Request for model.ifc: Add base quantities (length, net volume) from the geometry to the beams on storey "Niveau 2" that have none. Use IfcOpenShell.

First a look at what the model holds.

```python
import ifcopenshell
import ifcopenshell.util.element
import ifcopenshell.util.unit

model = ifcopenshell.open("model.ifc")
print(model.schema)
for unit_type in ("LENGTHUNIT", "AREAUNIT", "VOLUMEUNIT"):
    print(unit_type, ifcopenshell.util.unit.calculate_unit_scale(model, unit_type))
storey = next(s for s in model.by_type("IfcBuildingStorey") if s.Name == "Niveau 2")
beams = [e for e in ifcopenshell.util.element.get_decomposition(storey) if e.is_a("IfcBeam")]
for e in sorted(beams, key=lambda e: e.id()):
    print(e.id(), e.is_a(), e.Name, list(ifcopenshell.util.element.get_psets(e, qtos_only=True)), sep=" | ")
```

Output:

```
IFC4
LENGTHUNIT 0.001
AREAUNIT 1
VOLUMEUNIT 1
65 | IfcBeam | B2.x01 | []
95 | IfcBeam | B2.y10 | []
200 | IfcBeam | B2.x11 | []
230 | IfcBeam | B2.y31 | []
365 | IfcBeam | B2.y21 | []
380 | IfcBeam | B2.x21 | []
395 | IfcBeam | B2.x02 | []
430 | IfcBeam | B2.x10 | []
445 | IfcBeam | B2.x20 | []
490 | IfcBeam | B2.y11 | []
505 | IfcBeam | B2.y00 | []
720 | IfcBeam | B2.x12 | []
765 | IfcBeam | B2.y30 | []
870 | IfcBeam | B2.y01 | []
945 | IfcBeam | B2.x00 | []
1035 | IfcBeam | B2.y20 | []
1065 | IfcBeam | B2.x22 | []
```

```python
import ifcopenshell
import ifcopenshell.api.pset
import ifcopenshell.geom
import ifcopenshell.util.element
import ifcopenshell.util.shape
import ifcopenshell.util.unit

model = ifcopenshell.open("model.ifc")
unit_scale = ifcopenshell.util.unit.calculate_unit_scale(model)
volume_scale = ifcopenshell.util.unit.calculate_unit_scale(model, "VOLUMEUNIT")
settings = ifcopenshell.geom.settings()

storey = next(s for s in model.by_type("IfcBuildingStorey") if s.Name == "Niveau 2")
beams = [e for e in ifcopenshell.util.element.get_decomposition(storey) if e.is_a("IfcBeam")]

for e in sorted(beams, key=lambda e: e.id()):
    if ifcopenshell.util.element.get_psets(e, qtos_only=True, should_inherit=False):
        continue
    # Geometry comes back in metres, in the element's own axes.
    shape = ifcopenshell.geom.create_shape(settings, e)
    values = {
        "Length": ifcopenshell.util.shape.get_max_xyz(shape.geometry) / unit_scale,
        "NetVolume": ifcopenshell.util.shape.get_volume(shape.geometry) / volume_scale,
    }
    qto = ifcopenshell.api.pset.add_qto(model, product=e, name="Qto_BeamBaseQuantities")
    ifcopenshell.api.pset.edit_qto(model, qto=qto, properties=values)
    print(e.id(), {k: round(v, 3) for k, v in values.items()})

model.write("model_v2.ifc")
```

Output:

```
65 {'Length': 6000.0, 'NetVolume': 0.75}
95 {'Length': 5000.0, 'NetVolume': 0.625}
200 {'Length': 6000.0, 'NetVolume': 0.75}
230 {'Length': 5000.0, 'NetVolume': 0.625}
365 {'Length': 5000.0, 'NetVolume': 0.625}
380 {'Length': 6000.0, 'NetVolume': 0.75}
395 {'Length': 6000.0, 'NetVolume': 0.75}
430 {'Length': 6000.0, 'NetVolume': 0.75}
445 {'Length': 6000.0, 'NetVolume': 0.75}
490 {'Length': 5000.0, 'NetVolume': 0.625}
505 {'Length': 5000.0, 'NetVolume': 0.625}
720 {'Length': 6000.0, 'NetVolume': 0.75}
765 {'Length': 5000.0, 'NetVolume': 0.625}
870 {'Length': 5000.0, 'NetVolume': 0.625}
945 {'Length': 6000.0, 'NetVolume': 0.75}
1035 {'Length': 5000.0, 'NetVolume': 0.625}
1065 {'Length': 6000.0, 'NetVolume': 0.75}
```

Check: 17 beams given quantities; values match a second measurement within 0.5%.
